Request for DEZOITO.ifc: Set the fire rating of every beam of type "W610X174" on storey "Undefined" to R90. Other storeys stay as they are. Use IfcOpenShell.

First a look at what the model holds.

```python
import ifcopenshell
import ifcopenshell.util.element

model = ifcopenshell.open("DEZOITO.ifc")
print(model.schema)
storey = next(s for s in model.by_type("IfcBuildingStorey") if s.Name == "Undefined")
beams = [e for e in ifcopenshell.util.element.get_decomposition(storey) if e.is_a("IfcBeam")]
seen = {}
for e in beams:
    element_type = ifcopenshell.util.element.get_type(e)
    key = (element_type.Name if element_type != e and element_type else None, ifcopenshell.util.element.get_pset(e, "Pset_BeamCommon", "FireRating"))
    seen[key] = seen.get(key, 0) + 1
for (name, value), count in sorted(seen.items(), key=str):
    print(count, "x", name, "|", value)
```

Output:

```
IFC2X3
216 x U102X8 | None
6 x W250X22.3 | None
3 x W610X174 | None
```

```python
import ifcopenshell
import ifcopenshell.api.pset
import ifcopenshell.util.element

model = ifcopenshell.open("DEZOITO.ifc")

storey = next(s for s in model.by_type("IfcBuildingStorey") if s.Name == "Undefined")
beams = [e for e in ifcopenshell.util.element.get_decomposition(storey) if e.is_a("IfcBeam")]

count = 0
for e in beams:
    element_type = ifcopenshell.util.element.get_type(e)
    if element_type in (None, e) or element_type.Name != "W610X174":
        continue
    found = ifcopenshell.util.element.get_pset(e, "Pset_BeamCommon", should_inherit=False)
    if found:
        pset = model.by_id(found["id"])
        if len(ifcopenshell.util.element.get_elements_by_pset(pset)) > 1:
            pset = ifcopenshell.api.pset.unshare_pset(model, products=[e], pset=pset)[0]
    else:
        pset = ifcopenshell.api.pset.add_pset(model, product=e, name="Pset_BeamCommon")
    ifcopenshell.api.pset.edit_pset(model, pset=pset, properties={"FireRating": "R90"})
    count += 1

print(count, "beams updated")

model.write("DEZOITO_v2.ifc")
```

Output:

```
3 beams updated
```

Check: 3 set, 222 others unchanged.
